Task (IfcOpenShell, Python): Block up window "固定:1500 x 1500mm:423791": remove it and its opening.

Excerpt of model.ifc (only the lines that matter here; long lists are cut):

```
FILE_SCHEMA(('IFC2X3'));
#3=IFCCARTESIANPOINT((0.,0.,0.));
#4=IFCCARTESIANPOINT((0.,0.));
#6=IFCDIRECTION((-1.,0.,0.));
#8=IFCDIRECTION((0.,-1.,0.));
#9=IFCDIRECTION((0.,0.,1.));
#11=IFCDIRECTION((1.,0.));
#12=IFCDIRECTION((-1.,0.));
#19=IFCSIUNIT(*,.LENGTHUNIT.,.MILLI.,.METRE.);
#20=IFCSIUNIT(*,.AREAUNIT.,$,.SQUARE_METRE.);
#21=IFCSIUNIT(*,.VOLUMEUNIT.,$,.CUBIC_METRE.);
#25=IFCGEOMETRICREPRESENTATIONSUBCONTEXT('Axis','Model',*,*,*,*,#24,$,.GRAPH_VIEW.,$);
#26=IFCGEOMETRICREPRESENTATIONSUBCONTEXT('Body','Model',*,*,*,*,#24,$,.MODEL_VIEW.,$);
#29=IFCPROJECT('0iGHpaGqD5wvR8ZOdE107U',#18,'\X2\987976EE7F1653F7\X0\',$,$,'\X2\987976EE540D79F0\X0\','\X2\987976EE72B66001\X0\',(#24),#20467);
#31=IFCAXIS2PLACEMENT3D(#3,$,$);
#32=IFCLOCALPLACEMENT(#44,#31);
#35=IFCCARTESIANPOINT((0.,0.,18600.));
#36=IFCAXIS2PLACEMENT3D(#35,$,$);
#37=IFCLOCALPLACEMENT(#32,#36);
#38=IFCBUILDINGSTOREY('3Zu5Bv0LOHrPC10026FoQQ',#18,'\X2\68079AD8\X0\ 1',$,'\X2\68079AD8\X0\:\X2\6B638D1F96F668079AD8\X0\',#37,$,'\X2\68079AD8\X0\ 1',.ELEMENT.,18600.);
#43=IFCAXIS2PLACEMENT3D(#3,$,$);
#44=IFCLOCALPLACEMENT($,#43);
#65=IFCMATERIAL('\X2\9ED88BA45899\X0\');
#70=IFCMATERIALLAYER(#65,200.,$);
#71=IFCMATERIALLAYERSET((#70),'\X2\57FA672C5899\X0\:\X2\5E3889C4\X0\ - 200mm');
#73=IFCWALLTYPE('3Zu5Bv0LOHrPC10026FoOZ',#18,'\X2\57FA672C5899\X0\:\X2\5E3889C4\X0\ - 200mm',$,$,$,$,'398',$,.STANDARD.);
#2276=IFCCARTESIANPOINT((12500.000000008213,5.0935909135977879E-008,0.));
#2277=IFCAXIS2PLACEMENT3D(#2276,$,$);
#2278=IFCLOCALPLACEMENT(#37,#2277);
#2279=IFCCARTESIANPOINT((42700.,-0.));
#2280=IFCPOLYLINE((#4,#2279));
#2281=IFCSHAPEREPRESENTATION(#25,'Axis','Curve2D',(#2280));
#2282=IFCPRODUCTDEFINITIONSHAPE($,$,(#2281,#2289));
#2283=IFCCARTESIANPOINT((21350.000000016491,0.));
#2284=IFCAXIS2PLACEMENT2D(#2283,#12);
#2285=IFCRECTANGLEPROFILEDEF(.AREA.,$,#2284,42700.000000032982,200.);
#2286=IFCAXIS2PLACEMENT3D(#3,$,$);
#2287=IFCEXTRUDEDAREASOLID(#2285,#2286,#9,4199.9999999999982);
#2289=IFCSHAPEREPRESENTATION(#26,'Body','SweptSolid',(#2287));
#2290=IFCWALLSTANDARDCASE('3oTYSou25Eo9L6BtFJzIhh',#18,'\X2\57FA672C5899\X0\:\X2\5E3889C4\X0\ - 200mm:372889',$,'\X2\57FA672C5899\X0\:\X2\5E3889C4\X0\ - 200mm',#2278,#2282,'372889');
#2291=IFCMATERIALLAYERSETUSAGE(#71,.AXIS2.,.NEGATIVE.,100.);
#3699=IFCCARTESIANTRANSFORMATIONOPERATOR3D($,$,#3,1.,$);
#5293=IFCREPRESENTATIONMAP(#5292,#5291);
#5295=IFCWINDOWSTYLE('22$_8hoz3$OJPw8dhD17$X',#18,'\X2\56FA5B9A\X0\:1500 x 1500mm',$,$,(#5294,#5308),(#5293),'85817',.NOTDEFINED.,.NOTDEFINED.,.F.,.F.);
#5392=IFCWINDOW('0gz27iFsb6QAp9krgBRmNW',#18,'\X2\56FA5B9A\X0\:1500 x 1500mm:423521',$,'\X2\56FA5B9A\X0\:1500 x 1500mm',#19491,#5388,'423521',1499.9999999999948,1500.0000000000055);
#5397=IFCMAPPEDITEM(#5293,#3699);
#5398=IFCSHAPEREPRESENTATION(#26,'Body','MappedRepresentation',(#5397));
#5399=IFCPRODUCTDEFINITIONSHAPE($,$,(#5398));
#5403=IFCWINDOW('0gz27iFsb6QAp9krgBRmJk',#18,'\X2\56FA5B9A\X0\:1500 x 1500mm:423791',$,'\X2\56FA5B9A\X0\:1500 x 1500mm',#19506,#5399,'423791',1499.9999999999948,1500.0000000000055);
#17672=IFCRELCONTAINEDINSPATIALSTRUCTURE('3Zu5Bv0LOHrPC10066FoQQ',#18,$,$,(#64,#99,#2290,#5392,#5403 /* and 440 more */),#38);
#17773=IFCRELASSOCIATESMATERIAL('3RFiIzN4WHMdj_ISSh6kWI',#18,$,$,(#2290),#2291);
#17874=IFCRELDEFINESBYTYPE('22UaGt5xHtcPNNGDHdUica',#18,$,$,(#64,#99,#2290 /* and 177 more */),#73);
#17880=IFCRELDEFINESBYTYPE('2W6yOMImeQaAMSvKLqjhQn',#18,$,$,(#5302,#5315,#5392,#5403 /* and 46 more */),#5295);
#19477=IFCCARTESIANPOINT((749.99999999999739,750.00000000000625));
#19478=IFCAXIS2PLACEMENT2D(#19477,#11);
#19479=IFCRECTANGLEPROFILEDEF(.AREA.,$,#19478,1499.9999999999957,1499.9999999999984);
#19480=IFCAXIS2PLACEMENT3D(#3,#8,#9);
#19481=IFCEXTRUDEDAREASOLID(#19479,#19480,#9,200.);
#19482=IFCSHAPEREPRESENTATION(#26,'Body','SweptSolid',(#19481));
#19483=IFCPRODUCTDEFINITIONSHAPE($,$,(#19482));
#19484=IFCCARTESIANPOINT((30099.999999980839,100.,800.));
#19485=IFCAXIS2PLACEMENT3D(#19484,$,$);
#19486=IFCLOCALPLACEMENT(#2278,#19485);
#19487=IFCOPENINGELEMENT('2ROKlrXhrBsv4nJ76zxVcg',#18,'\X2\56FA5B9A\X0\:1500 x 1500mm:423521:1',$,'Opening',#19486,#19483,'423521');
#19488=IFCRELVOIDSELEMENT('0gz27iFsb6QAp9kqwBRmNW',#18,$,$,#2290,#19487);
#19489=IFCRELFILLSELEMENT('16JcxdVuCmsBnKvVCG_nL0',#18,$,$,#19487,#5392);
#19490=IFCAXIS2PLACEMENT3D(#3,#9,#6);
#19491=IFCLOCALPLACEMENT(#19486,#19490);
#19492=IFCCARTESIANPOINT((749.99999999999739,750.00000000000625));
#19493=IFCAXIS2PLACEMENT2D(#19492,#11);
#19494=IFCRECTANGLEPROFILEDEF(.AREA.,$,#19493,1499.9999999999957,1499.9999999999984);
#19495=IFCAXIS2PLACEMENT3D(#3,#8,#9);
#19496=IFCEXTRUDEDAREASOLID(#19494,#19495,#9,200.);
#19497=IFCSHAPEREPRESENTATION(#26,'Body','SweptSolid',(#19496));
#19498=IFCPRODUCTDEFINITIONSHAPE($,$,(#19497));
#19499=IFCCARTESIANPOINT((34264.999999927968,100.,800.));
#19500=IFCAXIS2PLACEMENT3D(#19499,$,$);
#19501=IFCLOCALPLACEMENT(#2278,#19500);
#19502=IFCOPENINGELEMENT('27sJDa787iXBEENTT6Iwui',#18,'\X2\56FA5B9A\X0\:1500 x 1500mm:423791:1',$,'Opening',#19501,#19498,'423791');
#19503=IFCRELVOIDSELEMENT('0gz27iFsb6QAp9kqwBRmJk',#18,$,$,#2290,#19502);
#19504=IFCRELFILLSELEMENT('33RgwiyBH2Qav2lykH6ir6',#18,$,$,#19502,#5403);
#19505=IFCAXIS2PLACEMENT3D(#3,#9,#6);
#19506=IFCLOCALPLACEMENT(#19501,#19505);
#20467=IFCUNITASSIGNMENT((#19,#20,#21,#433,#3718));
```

```python
import ifcopenshell
import ifcopenshell.api.feature
import ifcopenshell.api.root
import ifcopenshell.geom
import ifcopenshell.util.shape

model = ifcopenshell.open("model.ifc")
settings = ifcopenshell.geom.settings()


def volume(element):
    """Net volume in cubic metres, openings subtracted."""
    shape = ifcopenshell.geom.create_shape(settings, element)
    return ifcopenshell.util.shape.get_volume(shape.geometry)


window = model.by_guid("0gz27iFsb6QAp9krgBRmJk")
opening = window.FillsVoids[0].RelatingOpeningElement
wall = opening.VoidsElements[0].RelatingBuildingElement
before = volume(wall)

ifcopenshell.api.root.remove_product(model, product=window)
ifcopenshell.api.feature.remove_feature(model, feature=opening)

after = volume(wall)

print(f"wall volume {before:.3f} -> {after:.3f} m3")

model.write("model-out.ifc")
```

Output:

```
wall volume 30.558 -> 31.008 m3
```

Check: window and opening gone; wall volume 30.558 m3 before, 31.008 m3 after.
